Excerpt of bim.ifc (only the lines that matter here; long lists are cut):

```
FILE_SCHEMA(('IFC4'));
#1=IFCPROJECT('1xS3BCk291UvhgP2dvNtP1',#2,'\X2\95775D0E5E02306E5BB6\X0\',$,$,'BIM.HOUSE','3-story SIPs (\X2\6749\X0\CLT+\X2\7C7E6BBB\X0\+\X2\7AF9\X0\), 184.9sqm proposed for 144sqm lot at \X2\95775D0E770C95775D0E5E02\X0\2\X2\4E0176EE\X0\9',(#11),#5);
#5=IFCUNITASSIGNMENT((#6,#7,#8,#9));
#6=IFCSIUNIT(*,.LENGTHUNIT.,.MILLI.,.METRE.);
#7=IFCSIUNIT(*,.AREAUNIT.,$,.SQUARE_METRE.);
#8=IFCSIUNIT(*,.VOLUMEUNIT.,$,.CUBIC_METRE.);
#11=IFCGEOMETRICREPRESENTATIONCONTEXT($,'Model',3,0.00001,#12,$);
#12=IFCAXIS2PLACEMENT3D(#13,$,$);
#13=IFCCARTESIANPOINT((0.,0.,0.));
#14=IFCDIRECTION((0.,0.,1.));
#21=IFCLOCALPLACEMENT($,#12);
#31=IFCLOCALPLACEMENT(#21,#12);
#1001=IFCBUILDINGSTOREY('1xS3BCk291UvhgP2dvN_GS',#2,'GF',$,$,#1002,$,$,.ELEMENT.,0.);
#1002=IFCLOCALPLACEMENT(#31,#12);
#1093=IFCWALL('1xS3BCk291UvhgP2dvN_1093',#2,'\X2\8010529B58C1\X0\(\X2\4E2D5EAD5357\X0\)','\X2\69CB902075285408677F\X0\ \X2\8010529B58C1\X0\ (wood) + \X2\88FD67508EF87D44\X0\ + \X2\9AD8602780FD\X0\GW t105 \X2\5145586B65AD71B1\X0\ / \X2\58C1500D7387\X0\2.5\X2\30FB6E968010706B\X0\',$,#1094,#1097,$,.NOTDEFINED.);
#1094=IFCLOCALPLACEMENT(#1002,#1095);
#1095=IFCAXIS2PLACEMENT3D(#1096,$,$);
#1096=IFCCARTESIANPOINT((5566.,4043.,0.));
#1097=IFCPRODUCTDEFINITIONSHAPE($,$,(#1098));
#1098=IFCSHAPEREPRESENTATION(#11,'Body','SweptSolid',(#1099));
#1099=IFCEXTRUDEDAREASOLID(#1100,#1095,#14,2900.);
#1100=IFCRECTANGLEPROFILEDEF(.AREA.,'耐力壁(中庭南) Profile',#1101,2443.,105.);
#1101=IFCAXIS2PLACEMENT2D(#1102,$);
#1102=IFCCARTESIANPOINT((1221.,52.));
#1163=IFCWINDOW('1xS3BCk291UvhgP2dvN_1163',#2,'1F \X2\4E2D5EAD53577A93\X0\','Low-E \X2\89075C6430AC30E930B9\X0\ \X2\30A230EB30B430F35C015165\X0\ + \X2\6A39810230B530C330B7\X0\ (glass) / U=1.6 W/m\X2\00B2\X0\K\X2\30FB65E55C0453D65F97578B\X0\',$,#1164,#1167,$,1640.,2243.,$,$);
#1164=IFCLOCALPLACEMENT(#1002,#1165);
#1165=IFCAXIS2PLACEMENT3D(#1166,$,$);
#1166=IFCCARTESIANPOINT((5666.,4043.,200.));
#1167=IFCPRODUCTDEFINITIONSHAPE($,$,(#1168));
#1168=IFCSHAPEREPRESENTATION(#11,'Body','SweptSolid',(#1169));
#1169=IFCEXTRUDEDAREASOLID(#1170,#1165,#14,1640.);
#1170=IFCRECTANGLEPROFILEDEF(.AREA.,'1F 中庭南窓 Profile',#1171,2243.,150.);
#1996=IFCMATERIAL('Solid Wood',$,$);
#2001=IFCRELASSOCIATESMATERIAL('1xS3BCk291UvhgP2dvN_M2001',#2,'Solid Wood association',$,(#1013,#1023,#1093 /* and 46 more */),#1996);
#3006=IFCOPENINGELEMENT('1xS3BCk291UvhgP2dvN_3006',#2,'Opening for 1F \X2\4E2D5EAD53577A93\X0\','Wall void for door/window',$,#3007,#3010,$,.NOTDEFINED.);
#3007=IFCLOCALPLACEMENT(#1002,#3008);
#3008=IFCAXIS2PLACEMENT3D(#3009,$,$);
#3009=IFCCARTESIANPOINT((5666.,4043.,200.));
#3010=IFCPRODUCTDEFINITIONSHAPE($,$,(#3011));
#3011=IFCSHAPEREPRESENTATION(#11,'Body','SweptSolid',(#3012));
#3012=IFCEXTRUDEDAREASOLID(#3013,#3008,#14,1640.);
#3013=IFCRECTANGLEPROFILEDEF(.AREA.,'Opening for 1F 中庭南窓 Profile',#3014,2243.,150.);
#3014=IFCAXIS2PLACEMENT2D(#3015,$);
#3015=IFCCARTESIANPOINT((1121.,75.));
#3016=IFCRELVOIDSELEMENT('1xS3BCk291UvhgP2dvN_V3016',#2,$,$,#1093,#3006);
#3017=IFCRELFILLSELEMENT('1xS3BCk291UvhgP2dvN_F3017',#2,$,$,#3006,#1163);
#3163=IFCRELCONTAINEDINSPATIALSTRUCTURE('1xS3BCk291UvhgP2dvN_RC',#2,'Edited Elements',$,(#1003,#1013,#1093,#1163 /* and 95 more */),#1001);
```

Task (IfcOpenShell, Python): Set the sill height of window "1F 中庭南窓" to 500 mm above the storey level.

```python
import numpy as np
import ifcopenshell
import ifcopenshell.api.geometry
import ifcopenshell.geom
import ifcopenshell.util.element
import ifcopenshell.util.placement
import ifcopenshell.util.shape
import ifcopenshell.util.unit

model = ifcopenshell.open("bim.ifc")
unit_scale = ifcopenshell.util.unit.calculate_unit_scale(model)

window = model.by_id(1163)
opening = window.FillsVoids[0].RelatingOpeningElement
storey = ifcopenshell.util.element.get_container(window, ifc_class="IfcBuildingStorey")
level = ifcopenshell.util.placement.get_local_placement(storey.ObjectPlacement)[2, 3]

# The opening's origin need not be at the sill, so measure its lowest point.
shape = ifcopenshell.geom.create_shape(ifcopenshell.geom.settings(), opening)
bottom = ifcopenshell.util.shape.get_shape_bottom_elevation(shape, shape.geometry) / unit_scale
dz = level + 0.5 / unit_scale - bottom

shift = np.array([0.0, 0.0, dz])
# The window is not placed relative to its opening, so move both.
for product in (opening, window):
    matrix = ifcopenshell.util.placement.get_local_placement(product.ObjectPlacement)
    matrix[:3, 3] += shift
    ifcopenshell.api.geometry.edit_object_placement(model, product=product, matrix=matrix, is_si=False)

print(f"moved by {dz * unit_scale:+.3f} m")

model.write("bim_rev.ifc")
```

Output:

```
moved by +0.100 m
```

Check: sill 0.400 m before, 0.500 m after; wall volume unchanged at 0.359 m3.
